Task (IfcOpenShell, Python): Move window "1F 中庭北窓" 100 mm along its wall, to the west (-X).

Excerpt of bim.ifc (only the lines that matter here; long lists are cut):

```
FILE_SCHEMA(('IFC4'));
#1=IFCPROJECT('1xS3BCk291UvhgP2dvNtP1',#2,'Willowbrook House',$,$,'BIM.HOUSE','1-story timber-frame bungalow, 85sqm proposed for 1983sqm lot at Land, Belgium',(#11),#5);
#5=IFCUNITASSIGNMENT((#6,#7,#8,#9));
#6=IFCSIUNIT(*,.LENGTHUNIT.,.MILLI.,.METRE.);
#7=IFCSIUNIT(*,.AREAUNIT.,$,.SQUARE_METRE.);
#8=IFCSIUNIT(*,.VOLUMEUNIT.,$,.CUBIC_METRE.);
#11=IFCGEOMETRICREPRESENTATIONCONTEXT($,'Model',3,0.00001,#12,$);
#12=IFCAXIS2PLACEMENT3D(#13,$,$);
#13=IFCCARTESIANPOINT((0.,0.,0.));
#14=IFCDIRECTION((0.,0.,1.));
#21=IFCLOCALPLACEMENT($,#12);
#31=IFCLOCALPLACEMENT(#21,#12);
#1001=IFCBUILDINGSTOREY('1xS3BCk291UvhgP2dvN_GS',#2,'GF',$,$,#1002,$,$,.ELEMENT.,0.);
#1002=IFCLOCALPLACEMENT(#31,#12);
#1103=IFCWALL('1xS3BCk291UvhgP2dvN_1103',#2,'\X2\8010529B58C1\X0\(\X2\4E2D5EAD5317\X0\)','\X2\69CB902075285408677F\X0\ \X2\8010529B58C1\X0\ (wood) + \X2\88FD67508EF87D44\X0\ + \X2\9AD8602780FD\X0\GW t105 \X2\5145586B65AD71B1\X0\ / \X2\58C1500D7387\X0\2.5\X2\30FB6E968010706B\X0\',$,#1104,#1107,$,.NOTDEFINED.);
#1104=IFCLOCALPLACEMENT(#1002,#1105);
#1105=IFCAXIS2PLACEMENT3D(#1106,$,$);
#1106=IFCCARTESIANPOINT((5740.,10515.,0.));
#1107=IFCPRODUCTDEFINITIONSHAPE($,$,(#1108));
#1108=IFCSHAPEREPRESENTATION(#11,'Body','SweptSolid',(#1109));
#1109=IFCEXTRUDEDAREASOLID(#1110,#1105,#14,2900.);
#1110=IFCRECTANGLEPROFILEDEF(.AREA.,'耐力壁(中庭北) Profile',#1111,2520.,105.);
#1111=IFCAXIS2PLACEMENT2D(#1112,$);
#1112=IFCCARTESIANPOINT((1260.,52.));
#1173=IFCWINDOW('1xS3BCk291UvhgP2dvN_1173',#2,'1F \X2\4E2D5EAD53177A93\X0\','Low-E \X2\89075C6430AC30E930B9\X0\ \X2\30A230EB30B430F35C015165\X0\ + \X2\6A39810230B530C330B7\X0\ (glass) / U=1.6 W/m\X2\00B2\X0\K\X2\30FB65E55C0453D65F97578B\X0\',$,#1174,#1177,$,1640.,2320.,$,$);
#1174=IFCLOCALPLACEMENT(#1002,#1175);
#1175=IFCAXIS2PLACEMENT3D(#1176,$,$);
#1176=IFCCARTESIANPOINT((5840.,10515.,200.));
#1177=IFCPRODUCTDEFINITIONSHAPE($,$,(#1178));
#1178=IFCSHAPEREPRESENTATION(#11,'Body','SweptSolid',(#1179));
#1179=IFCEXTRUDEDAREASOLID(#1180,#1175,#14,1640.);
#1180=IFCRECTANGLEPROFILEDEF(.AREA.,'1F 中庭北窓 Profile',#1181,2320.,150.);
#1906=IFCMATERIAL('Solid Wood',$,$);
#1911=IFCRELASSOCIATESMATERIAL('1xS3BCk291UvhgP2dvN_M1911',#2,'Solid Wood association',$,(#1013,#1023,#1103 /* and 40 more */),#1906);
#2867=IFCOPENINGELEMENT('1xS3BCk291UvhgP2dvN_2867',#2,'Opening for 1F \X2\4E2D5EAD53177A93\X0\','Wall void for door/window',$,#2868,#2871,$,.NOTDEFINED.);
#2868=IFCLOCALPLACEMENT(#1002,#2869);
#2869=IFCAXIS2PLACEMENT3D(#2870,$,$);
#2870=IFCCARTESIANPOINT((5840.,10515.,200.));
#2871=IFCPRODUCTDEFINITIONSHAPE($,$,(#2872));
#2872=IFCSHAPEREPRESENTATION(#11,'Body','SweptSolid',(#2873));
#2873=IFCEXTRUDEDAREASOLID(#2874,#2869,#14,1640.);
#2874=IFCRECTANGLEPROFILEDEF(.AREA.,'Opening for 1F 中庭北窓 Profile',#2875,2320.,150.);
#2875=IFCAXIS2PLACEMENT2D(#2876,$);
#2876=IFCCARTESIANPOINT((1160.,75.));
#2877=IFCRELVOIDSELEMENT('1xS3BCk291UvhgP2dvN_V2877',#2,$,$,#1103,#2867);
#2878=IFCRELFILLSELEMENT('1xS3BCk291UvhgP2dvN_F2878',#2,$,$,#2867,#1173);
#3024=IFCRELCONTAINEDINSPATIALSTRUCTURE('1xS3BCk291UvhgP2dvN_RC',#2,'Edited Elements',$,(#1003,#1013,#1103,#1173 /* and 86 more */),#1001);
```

```python
import ifcopenshell
import ifcopenshell.api.geometry
import ifcopenshell.util.placement
import ifcopenshell.util.unit

model = ifcopenshell.open("bim.ifc")
unit_scale = ifcopenshell.util.unit.calculate_unit_scale(model)

window = model.by_id(1173)
opening = window.FillsVoids[0].RelatingOpeningElement
wall = opening.VoidsElements[0].RelatingBuildingElement

wall_matrix = ifcopenshell.util.placement.get_local_placement(wall.ObjectPlacement)
shift = wall_matrix[:3, 0] * -0.1 / unit_scale
before = ifcopenshell.util.placement.get_local_placement(window.ObjectPlacement)[:3, 3].copy()

# The window is not placed relative to its opening, so move both.
for product in (opening, window):
    matrix = ifcopenshell.util.placement.get_local_placement(product.ObjectPlacement)
    matrix[:3, 3] += shift
    ifcopenshell.api.geometry.edit_object_placement(model, product=product, matrix=matrix, is_si=False)

after = ifcopenshell.util.placement.get_local_placement(window.ObjectPlacement)[:3, 3]
print("window moved by", (after - before).round(3) + 0.0)

model.write("bim_updated.ifc")
```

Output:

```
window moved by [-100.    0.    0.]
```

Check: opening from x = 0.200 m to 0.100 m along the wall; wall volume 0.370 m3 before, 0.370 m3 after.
